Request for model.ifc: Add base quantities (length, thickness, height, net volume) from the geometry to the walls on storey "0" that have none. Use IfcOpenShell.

First a look at what the model holds.

```python
import ifcopenshell
import ifcopenshell.util.element
import ifcopenshell.util.unit

model = ifcopenshell.open("model.ifc")
print(model.schema)
for unit_type in ("LENGTHUNIT", "AREAUNIT", "VOLUMEUNIT"):
    print(unit_type, ifcopenshell.util.unit.calculate_unit_scale(model, unit_type))
storey = next(s for s in model.by_type("IfcBuildingStorey") if s.Name == "0")
walls = [e for e in ifcopenshell.util.element.get_decomposition(storey) if e.is_a("IfcWall")]
for e in sorted(walls, key=lambda e: e.id()):
    print(e.id(), e.is_a(), e.Name, list(ifcopenshell.util.element.get_psets(e, qtos_only=True)), sep=" | ")
```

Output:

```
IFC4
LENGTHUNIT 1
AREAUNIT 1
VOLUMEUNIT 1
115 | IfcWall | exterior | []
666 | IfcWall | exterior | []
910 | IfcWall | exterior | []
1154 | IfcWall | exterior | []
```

```python
import ifcopenshell
import ifcopenshell.api.pset
import ifcopenshell.geom
import ifcopenshell.util.element
import ifcopenshell.util.shape
import ifcopenshell.util.unit

model = ifcopenshell.open("model.ifc")
unit_scale = ifcopenshell.util.unit.calculate_unit_scale(model)
volume_scale = ifcopenshell.util.unit.calculate_unit_scale(model, "VOLUMEUNIT")
settings = ifcopenshell.geom.settings()

storey = next(s for s in model.by_type("IfcBuildingStorey") if s.Name == "0")
walls = [e for e in ifcopenshell.util.element.get_decomposition(storey) if e.is_a("IfcWall")]

for e in sorted(walls, key=lambda e: e.id()):
    if ifcopenshell.util.element.get_psets(e, qtos_only=True, should_inherit=False):
        continue
    # Geometry comes back in metres, in the element's own axes.
    shape = ifcopenshell.geom.create_shape(settings, e)
    values = {
        "Length": ifcopenshell.util.shape.get_x(shape.geometry) / unit_scale,
        "Width": ifcopenshell.util.shape.get_y(shape.geometry) / unit_scale,
        "Height": ifcopenshell.util.shape.get_z(shape.geometry) / unit_scale,
        "NetVolume": ifcopenshell.util.shape.get_volume(shape.geometry) / volume_scale,
    }
    qto = ifcopenshell.api.pset.add_qto(model, product=e, name="Qto_WallBaseQuantities")
    ifcopenshell.api.pset.edit_qto(model, qto=qto, properties=values)
    print(e.id(), {k: round(v, 3) for k, v in values.items()})

model.write("model_v2.ifc")
```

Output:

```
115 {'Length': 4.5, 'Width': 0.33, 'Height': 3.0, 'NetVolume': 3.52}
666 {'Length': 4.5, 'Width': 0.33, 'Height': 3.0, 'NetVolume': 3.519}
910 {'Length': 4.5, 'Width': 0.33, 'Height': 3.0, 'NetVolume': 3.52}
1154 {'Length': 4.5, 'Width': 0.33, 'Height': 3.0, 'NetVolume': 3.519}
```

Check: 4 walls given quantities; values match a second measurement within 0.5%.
